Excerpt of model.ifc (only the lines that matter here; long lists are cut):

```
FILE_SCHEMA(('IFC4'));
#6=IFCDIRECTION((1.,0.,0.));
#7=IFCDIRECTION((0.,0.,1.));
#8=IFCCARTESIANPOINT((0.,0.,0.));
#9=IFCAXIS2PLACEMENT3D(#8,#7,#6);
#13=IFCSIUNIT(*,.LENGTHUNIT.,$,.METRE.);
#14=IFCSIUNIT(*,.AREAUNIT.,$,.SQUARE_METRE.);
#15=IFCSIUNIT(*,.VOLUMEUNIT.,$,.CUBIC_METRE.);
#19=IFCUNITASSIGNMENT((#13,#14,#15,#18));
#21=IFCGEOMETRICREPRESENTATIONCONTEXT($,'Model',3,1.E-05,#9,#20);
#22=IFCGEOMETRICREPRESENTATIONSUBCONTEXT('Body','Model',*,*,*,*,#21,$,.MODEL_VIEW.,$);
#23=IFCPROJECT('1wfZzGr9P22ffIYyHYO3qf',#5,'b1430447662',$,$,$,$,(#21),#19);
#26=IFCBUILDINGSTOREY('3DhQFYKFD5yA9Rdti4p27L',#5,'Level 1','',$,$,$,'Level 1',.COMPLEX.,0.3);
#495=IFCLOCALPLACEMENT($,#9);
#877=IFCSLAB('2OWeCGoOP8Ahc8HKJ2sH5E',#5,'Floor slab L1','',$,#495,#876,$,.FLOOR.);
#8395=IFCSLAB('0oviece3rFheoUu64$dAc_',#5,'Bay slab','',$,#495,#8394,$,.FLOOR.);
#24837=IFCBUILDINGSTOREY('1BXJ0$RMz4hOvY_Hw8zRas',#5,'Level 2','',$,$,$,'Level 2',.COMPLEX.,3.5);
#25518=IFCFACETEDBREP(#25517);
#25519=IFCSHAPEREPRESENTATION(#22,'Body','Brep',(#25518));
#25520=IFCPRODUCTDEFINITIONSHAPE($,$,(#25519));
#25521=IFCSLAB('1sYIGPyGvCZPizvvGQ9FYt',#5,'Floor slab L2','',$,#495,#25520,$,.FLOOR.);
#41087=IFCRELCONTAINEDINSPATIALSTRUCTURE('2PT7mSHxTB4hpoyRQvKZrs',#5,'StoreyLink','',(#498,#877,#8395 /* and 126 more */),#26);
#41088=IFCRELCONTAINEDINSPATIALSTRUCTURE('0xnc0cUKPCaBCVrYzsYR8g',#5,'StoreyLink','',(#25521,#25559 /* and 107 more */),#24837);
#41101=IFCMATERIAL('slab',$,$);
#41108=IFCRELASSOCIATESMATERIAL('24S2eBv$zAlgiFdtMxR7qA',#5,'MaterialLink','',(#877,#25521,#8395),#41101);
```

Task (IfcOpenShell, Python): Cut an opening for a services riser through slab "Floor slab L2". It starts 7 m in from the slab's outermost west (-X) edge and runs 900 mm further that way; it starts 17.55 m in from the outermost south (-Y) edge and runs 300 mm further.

```python
import numpy as np
import ifcopenshell
import ifcopenshell.api.feature
import ifcopenshell.api.geometry
import ifcopenshell.api.root
import ifcopenshell.geom
import ifcopenshell.util.placement
import ifcopenshell.util.representation
import ifcopenshell.util.shape
import ifcopenshell.util.unit

model = ifcopenshell.open("model.ifc")
unit_scale = ifcopenshell.util.unit.calculate_unit_scale(model)
settings = ifcopenshell.geom.settings()


def volume(element):
    """Net volume in cubic metres, openings subtracted."""
    shape = ifcopenshell.geom.create_shape(settings, element)
    return ifcopenshell.util.shape.get_volume(shape.geometry)


slab = model.by_id(25521)
before = volume(slab)

# Extent in the slab's own axes, in metres. The edges named are its -X and -Y sides.
slab_shape = ifcopenshell.geom.create_shape(settings, slab)
vertices = ifcopenshell.util.shape.get_vertices(slab_shape.geometry)
x_min, y_min, bottom = vertices.min(axis=0)
top = vertices[:, 2].max()

opening = ifcopenshell.api.root.create_entity(model, ifc_class="IfcOpeningElement", name="Services riser opening", predefined_type="OPENING")
context = ifcopenshell.util.representation.get_context(model, "Model", "Body", "MODEL_VIEW")
width, depth = 0.9, 0.3
outline = [(0.0, 0.0), (width, 0.0), (width, depth), (0.0, depth), (0.0, 0.0)]
# Overshoot both faces by 50 mm so the cut is clean.
shape = ifcopenshell.api.geometry.add_slab_representation(
    model, context=context, depth=top - bottom + 0.1, polyline=outline
)
ifcopenshell.api.geometry.assign_representation(model, product=opening, representation=shape)

matrix = ifcopenshell.util.placement.get_local_placement(slab.ObjectPlacement)
matrix[:, 3] = matrix @ np.append(np.array([x_min + 7, y_min + 17.55, bottom - 0.05]) / unit_scale, 1.0)
ifcopenshell.api.geometry.edit_object_placement(model, product=opening, matrix=matrix, is_si=False)
ifcopenshell.api.feature.add_feature(model, feature=opening, element=slab)

after = volume(slab)

print(f"slab volume {before:.3f} -> {after:.3f} m3")

model.write("model_updated.ifc")
```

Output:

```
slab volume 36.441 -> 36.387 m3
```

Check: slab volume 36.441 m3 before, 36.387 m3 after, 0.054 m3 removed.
